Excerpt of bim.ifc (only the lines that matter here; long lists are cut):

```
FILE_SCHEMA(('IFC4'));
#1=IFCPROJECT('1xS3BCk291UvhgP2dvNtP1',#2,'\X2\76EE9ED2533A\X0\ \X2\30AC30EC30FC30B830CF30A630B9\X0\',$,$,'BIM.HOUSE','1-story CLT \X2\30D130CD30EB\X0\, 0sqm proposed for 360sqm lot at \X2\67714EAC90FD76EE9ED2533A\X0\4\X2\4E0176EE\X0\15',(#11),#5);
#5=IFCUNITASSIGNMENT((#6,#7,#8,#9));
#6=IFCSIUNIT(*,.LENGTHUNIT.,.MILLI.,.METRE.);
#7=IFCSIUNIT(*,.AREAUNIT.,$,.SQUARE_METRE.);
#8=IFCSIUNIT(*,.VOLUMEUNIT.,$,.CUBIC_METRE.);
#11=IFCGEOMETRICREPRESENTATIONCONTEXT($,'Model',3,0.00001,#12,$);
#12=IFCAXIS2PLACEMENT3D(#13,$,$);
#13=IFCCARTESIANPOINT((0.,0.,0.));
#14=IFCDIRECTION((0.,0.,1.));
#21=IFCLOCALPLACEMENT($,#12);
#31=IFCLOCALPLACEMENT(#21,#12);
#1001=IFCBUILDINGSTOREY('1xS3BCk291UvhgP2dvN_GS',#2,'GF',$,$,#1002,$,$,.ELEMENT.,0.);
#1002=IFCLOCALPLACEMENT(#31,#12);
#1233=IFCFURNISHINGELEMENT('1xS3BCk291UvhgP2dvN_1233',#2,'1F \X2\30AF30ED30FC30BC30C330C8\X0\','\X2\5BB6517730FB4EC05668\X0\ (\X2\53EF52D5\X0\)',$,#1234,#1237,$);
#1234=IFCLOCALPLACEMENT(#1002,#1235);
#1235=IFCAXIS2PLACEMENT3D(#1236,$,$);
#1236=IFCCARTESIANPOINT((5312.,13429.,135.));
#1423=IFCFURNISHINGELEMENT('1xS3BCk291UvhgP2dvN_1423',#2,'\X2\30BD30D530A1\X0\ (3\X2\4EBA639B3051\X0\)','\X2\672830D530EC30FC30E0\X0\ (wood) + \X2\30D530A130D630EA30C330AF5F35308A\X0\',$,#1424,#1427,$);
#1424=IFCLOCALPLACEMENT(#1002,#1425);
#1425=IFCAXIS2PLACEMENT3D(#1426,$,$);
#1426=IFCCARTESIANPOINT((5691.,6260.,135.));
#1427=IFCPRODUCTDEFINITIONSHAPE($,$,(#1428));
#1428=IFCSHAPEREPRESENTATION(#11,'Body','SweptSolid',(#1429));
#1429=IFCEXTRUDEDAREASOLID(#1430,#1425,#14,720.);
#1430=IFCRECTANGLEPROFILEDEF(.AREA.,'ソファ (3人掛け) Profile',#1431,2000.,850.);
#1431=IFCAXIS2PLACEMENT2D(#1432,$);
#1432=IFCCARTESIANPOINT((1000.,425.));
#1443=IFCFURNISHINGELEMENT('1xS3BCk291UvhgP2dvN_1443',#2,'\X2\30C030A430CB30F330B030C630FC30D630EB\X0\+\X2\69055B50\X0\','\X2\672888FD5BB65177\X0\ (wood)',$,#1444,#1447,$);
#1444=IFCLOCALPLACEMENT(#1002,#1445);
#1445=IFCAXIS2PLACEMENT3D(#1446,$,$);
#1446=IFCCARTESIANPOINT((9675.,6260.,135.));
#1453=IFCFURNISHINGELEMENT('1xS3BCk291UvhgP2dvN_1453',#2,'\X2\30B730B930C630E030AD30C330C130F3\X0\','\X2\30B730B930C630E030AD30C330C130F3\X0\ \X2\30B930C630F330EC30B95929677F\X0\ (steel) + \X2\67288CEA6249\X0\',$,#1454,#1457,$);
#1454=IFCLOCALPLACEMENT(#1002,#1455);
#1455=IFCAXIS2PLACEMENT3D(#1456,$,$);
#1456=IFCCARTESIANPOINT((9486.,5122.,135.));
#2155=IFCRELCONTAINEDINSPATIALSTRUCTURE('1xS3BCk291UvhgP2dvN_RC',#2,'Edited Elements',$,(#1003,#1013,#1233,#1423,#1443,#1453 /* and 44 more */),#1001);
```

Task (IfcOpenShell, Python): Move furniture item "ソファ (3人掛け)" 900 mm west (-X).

```python
import ifcopenshell
import ifcopenshell.api.geometry
import ifcopenshell.util.placement
import ifcopenshell.util.unit

model = ifcopenshell.open("bim.ifc")
unit_scale = ifcopenshell.util.unit.calculate_unit_scale(model)

item = model.by_id(1423)
matrix = ifcopenshell.util.placement.get_local_placement(item.ObjectPlacement)
matrix[0, 3] -= 0.9 / unit_scale
ifcopenshell.api.geometry.edit_object_placement(model, product=item, matrix=matrix, is_si=False)

print(ifcopenshell.util.placement.get_local_placement(item.ObjectPlacement).round(3) + 0.0)

model.write("bim_v2.ifc")
```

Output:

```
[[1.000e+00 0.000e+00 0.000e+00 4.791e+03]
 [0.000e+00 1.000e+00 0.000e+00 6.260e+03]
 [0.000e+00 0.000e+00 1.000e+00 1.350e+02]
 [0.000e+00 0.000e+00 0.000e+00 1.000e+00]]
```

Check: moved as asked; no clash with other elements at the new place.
